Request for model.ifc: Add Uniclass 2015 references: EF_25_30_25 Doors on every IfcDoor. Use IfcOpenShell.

First a look at what the model holds.

```python
import ifcopenshell

model = ifcopenshell.open("model.ifc")
print(model.schema)
print("classifications:", [c.Name for c in model.by_type("IfcClassification")])
for ifc_class in ("IfcDoor", "IfcRoof", "IfcStair", "IfcWall", "IfcWindow"):
    print(ifc_class, len(model.by_type(ifc_class)))
```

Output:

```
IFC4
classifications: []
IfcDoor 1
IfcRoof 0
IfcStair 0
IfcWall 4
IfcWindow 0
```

```python
import ifcopenshell
import ifcopenshell.api.classification

model = ifcopenshell.open("model.ifc")

system = ifcopenshell.api.classification.add_classification(model, classification="Uniclass 2015")

codes = {
    "IfcDoor": ("EF_25_30_25", "Doors"),
}
for ifc_class, (code, name) in codes.items():
    products = model.by_type(ifc_class)
    ifcopenshell.api.classification.add_reference(
        model, products=products, classification=system, identification=code, name=name
    )
    print(code, len(products))

model.write("model_v2.ifc")
```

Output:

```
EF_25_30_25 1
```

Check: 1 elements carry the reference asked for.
